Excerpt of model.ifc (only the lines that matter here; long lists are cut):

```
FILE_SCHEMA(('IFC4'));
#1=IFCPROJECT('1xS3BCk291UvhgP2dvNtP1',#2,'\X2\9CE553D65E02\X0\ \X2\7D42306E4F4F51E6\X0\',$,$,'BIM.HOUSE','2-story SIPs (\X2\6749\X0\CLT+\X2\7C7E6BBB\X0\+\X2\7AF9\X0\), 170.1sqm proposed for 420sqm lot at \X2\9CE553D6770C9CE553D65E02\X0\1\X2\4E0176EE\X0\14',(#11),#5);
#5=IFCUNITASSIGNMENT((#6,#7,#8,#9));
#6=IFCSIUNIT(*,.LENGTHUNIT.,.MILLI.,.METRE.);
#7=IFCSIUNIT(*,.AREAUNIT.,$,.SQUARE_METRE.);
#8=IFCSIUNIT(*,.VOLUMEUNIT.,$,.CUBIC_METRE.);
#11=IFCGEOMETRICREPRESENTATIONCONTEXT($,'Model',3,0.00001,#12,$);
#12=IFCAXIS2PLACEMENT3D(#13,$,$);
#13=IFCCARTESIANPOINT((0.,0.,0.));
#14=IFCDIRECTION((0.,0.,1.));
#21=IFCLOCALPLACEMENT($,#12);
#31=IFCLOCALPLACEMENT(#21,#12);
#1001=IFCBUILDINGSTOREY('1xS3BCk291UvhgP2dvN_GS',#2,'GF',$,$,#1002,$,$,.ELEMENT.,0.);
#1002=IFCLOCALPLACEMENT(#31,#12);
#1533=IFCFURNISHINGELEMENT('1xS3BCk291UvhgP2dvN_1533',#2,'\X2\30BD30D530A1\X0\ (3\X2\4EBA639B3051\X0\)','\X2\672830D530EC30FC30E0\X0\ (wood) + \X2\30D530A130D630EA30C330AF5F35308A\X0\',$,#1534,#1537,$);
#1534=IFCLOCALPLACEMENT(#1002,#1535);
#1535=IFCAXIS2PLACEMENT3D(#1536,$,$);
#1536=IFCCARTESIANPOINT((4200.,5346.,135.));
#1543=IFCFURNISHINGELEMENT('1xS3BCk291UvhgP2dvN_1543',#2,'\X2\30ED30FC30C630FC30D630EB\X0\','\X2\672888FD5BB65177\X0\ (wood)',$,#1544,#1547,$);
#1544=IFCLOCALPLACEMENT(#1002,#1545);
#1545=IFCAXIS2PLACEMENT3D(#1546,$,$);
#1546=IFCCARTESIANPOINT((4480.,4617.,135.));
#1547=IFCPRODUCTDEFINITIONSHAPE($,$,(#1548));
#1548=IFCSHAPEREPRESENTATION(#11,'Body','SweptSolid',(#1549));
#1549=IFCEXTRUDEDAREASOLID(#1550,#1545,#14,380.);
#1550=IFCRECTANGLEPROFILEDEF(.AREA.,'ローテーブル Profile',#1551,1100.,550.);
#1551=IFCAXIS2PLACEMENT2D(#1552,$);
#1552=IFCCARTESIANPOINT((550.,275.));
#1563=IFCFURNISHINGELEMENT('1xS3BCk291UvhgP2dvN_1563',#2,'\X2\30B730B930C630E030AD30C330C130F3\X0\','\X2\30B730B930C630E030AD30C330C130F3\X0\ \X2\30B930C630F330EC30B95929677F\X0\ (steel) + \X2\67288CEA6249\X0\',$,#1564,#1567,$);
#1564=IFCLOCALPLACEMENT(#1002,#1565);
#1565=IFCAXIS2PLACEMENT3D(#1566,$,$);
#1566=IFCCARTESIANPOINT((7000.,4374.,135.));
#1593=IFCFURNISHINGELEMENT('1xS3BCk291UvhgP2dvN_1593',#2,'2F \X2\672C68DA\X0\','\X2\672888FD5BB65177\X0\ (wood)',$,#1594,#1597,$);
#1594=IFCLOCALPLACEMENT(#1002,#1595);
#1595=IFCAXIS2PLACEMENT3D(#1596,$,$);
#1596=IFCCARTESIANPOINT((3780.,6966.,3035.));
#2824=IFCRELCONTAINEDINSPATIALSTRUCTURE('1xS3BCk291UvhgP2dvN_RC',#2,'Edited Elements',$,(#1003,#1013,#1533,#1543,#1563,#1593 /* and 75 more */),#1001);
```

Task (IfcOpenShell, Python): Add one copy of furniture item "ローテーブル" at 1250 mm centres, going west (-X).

```python
import numpy as np
import ifcopenshell
import ifcopenshell.api.geometry
import ifcopenshell.api.root
import ifcopenshell.util.element
import ifcopenshell.util.placement
import ifcopenshell.util.unit

model = ifcopenshell.open("model.ifc")
unit_scale = ifcopenshell.util.unit.calculate_unit_scale(model)


def reuse_history(source, copy):
    """copy_class also copies each property set's owner history, people and application; keep the originals."""
    for rel in copy.IsDefinedBy:
        if rel.is_a("IfcRelDefinesByProperties") and (history := rel.RelatingPropertyDefinition.OwnerHistory):
            rel.RelatingPropertyDefinition.OwnerHistory = source.OwnerHistory
            ifcopenshell.util.element.remove_deep2(model, history)


source = model.by_id(1543)
base = ifcopenshell.util.placement.get_local_placement(source.ObjectPlacement)
step = np.array([-1.0, 0.0, 0.0]) * 1.25 / unit_scale

for i in range(1, 2):
    copy = ifcopenshell.api.root.copy_class(model, product=source)
    copy.Representation = ifcopenshell.util.element.copy_deep(
        model, source.Representation, exclude=["IfcGeometricRepresentationContext", "IfcRepresentationMap"]
    )
    reuse_history(source, copy)
    matrix = base.copy()
    matrix[:3, 3] += i * step
    print("added at", matrix[:3, 3].round(3) + 0.0)
    ifcopenshell.api.geometry.edit_object_placement(model, product=copy, matrix=matrix, is_si=False)

model.write("model_rev.ifc")
```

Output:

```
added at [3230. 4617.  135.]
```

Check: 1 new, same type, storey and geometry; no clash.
